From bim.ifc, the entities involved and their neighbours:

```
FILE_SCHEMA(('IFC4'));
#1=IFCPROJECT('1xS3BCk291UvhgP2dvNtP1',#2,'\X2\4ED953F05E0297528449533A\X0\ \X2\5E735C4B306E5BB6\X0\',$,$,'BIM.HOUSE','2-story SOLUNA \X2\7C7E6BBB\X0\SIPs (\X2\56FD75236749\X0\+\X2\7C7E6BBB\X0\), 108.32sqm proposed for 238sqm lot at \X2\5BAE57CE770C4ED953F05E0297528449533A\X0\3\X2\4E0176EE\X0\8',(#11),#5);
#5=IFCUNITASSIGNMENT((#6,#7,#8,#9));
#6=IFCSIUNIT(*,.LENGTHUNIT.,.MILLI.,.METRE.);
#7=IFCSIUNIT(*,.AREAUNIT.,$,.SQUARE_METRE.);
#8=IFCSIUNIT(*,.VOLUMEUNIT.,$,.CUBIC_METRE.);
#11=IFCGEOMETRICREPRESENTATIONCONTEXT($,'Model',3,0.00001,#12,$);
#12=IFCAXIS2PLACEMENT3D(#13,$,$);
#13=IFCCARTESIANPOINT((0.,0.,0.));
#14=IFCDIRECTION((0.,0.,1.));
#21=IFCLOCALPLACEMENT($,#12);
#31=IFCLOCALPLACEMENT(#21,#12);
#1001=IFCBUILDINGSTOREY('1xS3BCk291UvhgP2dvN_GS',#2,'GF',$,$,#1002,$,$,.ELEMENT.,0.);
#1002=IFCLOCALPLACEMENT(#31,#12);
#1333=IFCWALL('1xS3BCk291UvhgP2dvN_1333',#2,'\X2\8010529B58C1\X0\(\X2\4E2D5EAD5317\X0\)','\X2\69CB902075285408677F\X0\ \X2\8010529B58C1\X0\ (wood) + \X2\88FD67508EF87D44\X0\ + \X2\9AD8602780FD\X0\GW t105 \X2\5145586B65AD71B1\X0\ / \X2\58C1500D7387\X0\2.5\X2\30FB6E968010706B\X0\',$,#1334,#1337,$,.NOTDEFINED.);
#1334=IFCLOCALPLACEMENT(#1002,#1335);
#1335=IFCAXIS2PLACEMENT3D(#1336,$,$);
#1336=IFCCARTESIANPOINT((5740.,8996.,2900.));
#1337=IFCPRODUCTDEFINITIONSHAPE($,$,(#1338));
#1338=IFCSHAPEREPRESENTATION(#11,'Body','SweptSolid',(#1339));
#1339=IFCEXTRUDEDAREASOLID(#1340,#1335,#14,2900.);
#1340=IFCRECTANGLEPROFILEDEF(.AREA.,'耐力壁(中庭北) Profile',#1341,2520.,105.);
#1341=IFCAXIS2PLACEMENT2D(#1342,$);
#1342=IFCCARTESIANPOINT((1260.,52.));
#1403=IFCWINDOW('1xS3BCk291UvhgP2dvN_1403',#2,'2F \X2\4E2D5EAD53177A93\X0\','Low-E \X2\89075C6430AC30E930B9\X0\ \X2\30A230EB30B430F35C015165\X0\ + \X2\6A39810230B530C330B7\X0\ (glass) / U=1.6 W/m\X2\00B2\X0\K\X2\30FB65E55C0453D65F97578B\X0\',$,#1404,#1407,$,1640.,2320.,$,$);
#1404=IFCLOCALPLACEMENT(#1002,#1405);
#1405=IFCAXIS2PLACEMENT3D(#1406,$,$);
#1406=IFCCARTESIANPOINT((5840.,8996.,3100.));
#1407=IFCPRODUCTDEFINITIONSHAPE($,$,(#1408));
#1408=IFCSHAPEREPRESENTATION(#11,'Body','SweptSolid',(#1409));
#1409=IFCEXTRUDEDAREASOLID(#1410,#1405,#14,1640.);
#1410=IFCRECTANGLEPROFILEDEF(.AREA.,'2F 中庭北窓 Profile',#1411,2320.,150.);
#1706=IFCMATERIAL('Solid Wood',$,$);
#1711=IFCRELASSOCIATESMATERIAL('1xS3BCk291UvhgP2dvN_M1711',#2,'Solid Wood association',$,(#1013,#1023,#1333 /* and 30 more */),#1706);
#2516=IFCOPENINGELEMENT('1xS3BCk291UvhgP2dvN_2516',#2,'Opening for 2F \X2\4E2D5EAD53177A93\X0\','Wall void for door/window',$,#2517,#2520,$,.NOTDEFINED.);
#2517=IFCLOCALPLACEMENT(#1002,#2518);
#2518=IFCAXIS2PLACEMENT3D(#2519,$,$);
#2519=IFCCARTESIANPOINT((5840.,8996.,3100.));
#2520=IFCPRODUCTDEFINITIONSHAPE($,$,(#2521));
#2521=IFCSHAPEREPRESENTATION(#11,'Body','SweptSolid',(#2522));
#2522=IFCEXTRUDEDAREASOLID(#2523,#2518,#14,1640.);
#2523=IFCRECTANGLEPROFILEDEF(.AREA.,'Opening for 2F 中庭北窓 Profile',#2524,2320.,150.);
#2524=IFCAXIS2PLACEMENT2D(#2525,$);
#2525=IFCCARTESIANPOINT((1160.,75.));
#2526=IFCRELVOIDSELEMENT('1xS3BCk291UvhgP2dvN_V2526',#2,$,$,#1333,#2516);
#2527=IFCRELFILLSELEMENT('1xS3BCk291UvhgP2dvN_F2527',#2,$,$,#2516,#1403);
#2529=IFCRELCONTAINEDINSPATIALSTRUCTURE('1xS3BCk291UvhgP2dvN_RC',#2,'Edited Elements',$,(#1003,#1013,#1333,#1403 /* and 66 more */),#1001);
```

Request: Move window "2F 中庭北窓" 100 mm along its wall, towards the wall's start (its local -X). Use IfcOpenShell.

```python
import ifcopenshell
import ifcopenshell.api.geometry
import ifcopenshell.util.placement
import ifcopenshell.util.unit

model = ifcopenshell.open("bim.ifc")
unit_scale = ifcopenshell.util.unit.calculate_unit_scale(model)

window = model.by_guid("1xS3BCk291UvhgP2dvN_1403")
opening = window.FillsVoids[0].RelatingOpeningElement
wall = opening.VoidsElements[0].RelatingBuildingElement

wall_matrix = ifcopenshell.util.placement.get_local_placement(wall.ObjectPlacement)
shift = wall_matrix[:3, 0] * -0.1 / unit_scale
before = ifcopenshell.util.placement.get_local_placement(window.ObjectPlacement)[:3, 3].copy()

# The window is not placed relative to its opening, so move both.
for product in (opening, window):
    matrix = ifcopenshell.util.placement.get_local_placement(product.ObjectPlacement)
    matrix[:3, 3] += shift
    ifcopenshell.api.geometry.edit_object_placement(model, product=product, matrix=matrix, is_si=False)

after = ifcopenshell.util.placement.get_local_placement(window.ObjectPlacement)[:3, 3]
print("window moved by", (after - before).round(3) + 0.0)

model.write("bim_edited.ifc")
```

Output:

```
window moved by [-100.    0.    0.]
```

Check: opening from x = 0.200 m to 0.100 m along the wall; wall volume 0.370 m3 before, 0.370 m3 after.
